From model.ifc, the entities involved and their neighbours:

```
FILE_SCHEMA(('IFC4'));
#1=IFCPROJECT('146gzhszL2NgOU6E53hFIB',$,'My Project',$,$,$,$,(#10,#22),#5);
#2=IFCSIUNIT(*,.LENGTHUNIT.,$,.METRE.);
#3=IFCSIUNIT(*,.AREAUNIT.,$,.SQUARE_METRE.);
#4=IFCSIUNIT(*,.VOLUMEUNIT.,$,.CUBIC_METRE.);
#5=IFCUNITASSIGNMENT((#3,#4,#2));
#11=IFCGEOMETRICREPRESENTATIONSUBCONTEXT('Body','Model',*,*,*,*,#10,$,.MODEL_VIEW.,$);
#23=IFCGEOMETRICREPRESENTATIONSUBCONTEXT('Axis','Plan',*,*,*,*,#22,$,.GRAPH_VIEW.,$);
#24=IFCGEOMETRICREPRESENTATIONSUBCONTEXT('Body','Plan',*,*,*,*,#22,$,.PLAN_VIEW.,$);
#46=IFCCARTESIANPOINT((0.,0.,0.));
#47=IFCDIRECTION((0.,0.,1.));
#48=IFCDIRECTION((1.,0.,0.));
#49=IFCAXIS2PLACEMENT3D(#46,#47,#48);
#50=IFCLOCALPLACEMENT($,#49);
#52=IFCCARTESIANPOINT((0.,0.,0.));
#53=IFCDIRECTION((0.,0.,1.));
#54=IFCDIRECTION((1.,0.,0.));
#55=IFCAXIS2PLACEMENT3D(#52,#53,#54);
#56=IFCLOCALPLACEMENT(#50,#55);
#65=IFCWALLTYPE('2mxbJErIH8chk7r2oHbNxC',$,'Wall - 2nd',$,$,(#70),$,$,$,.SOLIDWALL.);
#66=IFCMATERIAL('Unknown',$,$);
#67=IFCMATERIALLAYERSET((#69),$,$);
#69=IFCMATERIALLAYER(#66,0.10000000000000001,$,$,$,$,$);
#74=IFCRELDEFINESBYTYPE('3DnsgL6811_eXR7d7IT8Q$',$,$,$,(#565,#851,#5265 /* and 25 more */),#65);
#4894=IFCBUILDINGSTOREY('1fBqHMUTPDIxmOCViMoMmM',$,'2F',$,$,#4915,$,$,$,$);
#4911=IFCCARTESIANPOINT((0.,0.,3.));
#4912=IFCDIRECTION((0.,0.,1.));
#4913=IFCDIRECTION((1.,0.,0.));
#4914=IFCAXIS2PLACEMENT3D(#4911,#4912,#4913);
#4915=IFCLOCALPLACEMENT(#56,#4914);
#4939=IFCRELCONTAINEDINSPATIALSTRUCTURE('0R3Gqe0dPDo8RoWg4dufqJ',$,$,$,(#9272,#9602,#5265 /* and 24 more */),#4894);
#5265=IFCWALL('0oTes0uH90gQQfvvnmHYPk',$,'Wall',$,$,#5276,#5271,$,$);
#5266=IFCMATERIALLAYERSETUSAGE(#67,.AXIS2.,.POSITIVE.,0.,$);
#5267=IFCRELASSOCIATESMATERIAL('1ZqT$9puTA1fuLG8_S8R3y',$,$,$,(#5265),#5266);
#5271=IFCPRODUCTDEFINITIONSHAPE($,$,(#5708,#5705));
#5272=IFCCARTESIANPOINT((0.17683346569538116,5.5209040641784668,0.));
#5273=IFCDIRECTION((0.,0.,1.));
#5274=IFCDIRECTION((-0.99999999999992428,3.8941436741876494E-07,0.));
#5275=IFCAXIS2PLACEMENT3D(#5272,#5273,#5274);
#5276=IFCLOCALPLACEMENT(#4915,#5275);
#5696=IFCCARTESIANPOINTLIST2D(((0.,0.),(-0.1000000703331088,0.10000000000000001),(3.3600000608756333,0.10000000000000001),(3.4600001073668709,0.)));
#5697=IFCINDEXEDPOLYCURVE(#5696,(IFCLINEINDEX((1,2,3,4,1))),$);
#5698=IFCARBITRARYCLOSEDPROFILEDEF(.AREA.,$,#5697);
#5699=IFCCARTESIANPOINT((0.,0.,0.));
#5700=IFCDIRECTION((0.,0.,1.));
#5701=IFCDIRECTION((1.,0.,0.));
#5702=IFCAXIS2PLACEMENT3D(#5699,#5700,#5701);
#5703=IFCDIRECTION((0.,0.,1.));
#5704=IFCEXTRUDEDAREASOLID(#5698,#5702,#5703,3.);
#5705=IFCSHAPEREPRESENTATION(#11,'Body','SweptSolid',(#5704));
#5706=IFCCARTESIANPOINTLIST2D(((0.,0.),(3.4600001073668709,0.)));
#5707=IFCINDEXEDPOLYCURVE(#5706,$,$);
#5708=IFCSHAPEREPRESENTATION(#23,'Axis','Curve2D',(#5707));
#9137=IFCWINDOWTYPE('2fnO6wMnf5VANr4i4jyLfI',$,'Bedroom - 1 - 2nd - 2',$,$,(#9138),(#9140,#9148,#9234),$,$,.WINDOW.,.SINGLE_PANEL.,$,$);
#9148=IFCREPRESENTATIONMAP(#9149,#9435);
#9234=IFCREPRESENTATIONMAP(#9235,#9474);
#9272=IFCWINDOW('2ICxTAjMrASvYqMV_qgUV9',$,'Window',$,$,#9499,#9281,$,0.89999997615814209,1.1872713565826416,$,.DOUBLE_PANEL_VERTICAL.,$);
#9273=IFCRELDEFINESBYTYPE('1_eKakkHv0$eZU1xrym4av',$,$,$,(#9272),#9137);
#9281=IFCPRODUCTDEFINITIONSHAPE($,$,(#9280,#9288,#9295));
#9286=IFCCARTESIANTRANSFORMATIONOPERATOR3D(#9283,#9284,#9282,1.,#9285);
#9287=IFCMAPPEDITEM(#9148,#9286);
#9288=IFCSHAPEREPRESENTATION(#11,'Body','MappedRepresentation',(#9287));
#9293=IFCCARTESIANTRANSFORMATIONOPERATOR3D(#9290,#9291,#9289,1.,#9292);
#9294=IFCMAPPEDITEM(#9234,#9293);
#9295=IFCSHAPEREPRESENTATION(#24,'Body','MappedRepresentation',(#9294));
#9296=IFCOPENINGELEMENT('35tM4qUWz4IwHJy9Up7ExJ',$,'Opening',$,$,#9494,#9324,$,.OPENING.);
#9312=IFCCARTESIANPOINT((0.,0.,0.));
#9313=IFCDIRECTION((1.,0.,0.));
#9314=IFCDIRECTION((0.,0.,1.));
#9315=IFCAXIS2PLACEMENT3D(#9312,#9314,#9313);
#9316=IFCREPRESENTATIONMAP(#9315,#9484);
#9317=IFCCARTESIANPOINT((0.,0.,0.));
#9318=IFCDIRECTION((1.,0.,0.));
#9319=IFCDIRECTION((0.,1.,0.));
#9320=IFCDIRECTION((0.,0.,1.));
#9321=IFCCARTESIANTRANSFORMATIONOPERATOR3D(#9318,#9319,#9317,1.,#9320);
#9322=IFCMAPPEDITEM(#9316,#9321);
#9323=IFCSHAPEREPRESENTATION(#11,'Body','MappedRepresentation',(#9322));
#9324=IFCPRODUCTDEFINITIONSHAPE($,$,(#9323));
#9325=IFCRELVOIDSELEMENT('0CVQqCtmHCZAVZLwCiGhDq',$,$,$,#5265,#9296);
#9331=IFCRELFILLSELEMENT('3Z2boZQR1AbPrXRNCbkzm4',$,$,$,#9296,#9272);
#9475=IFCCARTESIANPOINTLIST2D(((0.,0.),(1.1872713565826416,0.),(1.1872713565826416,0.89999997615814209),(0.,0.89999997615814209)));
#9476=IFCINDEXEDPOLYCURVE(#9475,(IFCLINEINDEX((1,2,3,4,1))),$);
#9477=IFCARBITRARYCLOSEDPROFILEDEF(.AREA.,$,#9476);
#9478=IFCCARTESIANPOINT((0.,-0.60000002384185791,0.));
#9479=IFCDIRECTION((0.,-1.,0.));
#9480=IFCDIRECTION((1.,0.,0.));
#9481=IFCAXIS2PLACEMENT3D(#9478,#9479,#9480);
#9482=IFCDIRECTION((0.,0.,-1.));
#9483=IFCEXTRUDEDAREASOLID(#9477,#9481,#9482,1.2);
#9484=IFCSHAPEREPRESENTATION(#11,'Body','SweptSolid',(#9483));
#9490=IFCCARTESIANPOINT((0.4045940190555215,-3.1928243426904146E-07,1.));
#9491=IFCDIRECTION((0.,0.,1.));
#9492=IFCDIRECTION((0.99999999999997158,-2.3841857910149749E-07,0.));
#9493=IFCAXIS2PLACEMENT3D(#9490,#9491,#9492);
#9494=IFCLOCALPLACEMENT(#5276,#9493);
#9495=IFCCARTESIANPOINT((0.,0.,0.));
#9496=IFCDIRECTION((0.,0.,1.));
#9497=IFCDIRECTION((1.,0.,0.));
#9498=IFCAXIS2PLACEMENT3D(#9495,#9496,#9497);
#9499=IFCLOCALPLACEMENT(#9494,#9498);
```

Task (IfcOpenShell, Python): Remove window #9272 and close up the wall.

```python
import ifcopenshell
import ifcopenshell.api.feature
import ifcopenshell.api.root
import ifcopenshell.geom
import ifcopenshell.util.shape

model = ifcopenshell.open("model.ifc")
settings = ifcopenshell.geom.settings()


def volume(element):
    """Net volume in cubic metres, openings subtracted."""
    shape = ifcopenshell.geom.create_shape(settings, element)
    return ifcopenshell.util.shape.get_volume(shape.geometry)


window = model.by_guid("2ICxTAjMrASvYqMV_qgUV9")
opening = window.FillsVoids[0].RelatingOpeningElement
wall = opening.VoidsElements[0].RelatingBuildingElement
before = volume(wall)

ifcopenshell.api.root.remove_product(model, product=window)
ifcopenshell.api.feature.remove_feature(model, feature=opening)

after = volume(wall)

print(f"wall volume {before:.3f} -> {after:.3f} m3")

model.write("model_v2.ifc")
```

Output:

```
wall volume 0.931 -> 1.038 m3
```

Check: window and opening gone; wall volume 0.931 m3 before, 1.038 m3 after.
